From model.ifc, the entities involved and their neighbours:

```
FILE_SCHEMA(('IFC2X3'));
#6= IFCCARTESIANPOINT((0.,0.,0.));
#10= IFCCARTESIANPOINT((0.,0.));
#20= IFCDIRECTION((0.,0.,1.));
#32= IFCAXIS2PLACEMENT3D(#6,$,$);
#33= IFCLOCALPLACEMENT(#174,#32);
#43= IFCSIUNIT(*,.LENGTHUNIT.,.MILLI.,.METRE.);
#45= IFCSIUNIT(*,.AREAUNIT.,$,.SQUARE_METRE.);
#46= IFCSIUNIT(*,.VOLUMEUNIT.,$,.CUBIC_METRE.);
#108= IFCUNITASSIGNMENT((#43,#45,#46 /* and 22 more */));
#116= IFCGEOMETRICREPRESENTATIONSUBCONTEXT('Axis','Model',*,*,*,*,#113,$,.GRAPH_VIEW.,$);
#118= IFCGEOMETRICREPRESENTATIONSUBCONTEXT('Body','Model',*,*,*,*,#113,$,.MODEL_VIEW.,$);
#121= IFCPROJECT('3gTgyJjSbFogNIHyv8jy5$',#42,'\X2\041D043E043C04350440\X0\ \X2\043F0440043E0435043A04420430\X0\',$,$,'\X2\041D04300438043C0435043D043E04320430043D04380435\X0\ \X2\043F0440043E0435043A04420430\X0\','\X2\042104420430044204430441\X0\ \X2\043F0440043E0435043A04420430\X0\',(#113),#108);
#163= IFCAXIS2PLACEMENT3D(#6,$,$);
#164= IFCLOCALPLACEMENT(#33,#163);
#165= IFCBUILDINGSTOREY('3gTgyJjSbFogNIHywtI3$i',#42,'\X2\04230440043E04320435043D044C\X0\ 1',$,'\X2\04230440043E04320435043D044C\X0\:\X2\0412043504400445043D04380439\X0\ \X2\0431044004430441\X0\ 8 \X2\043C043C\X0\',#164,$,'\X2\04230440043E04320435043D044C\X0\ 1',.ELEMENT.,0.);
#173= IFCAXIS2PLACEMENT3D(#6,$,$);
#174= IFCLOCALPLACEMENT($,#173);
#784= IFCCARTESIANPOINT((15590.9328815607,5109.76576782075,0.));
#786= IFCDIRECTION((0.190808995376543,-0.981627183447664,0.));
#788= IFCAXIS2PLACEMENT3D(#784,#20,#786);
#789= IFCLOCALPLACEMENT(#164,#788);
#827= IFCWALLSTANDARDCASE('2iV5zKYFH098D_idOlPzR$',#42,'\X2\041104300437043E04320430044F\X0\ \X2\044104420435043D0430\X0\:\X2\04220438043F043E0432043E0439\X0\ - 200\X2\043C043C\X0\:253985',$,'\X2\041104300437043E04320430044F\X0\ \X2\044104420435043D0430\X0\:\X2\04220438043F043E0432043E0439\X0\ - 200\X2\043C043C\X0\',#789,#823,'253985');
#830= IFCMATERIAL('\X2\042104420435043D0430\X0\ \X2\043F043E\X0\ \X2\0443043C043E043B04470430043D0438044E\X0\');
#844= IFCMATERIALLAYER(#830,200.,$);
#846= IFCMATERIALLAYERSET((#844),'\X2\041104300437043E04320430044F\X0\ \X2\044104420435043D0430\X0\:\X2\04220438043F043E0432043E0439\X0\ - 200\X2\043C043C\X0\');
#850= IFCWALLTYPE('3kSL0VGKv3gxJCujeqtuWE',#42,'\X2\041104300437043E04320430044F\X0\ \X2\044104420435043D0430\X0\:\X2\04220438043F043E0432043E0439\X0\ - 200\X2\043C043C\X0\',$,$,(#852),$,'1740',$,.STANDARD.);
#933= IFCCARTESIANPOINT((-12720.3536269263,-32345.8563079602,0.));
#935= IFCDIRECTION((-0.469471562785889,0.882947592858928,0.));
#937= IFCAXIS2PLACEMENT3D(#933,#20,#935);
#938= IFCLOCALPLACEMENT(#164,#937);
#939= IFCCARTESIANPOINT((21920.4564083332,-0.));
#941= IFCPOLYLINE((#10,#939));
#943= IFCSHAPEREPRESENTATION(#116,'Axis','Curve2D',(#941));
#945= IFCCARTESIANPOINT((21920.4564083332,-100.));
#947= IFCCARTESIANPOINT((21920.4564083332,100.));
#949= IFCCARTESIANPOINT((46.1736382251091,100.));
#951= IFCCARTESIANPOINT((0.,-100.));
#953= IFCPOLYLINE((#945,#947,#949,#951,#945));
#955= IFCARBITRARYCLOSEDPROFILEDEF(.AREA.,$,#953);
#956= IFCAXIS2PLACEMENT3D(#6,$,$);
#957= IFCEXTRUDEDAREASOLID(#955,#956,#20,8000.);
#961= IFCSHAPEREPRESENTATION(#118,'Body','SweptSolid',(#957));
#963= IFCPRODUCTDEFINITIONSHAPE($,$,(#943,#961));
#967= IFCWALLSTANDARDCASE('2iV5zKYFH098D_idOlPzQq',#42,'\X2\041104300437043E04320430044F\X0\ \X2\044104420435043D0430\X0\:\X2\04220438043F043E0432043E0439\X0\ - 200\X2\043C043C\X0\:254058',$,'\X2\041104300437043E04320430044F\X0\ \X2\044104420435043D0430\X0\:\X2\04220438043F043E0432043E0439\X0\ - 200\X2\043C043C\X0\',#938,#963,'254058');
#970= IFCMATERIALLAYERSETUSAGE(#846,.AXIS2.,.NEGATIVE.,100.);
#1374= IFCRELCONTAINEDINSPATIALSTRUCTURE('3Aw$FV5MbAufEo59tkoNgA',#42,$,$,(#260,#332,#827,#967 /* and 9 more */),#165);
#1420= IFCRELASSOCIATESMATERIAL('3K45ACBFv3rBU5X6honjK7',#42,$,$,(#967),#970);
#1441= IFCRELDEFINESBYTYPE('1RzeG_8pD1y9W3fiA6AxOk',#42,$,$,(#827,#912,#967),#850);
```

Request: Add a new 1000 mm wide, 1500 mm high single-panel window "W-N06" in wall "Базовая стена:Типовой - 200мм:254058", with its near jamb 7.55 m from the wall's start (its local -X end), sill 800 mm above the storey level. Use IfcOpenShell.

```python
import numpy as np
import ifcopenshell
import ifcopenshell.api.feature
import ifcopenshell.api.geometry
import ifcopenshell.api.root
import ifcopenshell.api.spatial
import ifcopenshell.api.type
import ifcopenshell.geom
import ifcopenshell.util.element
import ifcopenshell.util.placement
import ifcopenshell.util.representation
import ifcopenshell.util.shape
import ifcopenshell.util.unit

model = ifcopenshell.open("model.ifc")
unit_scale = ifcopenshell.util.unit.calculate_unit_scale(model)
settings = ifcopenshell.geom.settings()


def volume(element):
    """Net volume in cubic metres, openings subtracted."""
    shape = ifcopenshell.geom.create_shape(settings, element)
    return ifcopenshell.util.shape.get_volume(shape.geometry)


wall = model.by_guid("2iV5zKYFH098D_idOlPzQq")
storey = ifcopenshell.util.element.get_container(wall, ifc_class="IfcBuildingStorey")
context = ifcopenshell.util.representation.get_context(model, "Model", "Body", "MODEL_VIEW")
before = volume(wall)

width, height, from_end, sill = 1, 1.5, 7.55, 0.8  # metres

# The wall runs along its own X axis, and the end named is its -X end.
wall_shape = ifcopenshell.geom.create_shape(settings, wall)
x, y, z = ifcopenshell.util.shape.get_vertices(wall_shape.geometry).T
start = x.min() + from_end
face, thickness = float(y.min()), float(y.max() - y.min())
wall_matrix = ifcopenshell.util.placement.get_local_placement(wall.ObjectPlacement)
level = ifcopenshell.util.placement.get_local_placement(storey.ObjectPlacement)[2, 3]


def in_wall(x, y):
    """Placement at x, y metres in the wall's axes, at sill height."""
    matrix = wall_matrix.copy()
    matrix[:, 3] = wall_matrix @ np.array([x / unit_scale, y / unit_scale, 0.0, 1.0])
    matrix[2, 3] = level + sill / unit_scale
    return matrix


# Opening: a box that overshoots both wall faces by 50 mm.
opening = ifcopenshell.api.root.create_entity(model, ifc_class="IfcOpeningElement")
box = ifcopenshell.api.geometry.add_wall_representation(
    model, context=context, length=width, height=height, thickness=thickness + 0.1
)
ifcopenshell.api.geometry.assign_representation(model, product=opening, representation=box)
ifcopenshell.api.geometry.edit_object_placement(model, product=opening, matrix=in_wall(start, face - 0.05), is_si=False)
ifcopenshell.api.feature.add_feature(model, feature=opening, element=wall)

window = ifcopenshell.api.root.create_entity(model, ifc_class="IfcWindow", name="W-N06")
window.OverallWidth, window.OverallHeight = width / unit_scale, height / unit_scale
body = ifcopenshell.api.geometry.add_window_representation(
    model,
    context=context,
    overall_width=window.OverallWidth,
    overall_height=window.OverallHeight,
    partition_type="SINGLE_PANEL",
)
ifcopenshell.api.geometry.assign_representation(model, product=window, representation=body)
ifcopenshell.api.spatial.assign_container(model, products=[window], relating_structure=storey)
fills = ifcopenshell.api.feature.add_filling(model, opening=opening, element=window)
fills.OwnerHistory = window.OwnerHistory  # required in IFC2X3

# IFC2X3 keeps the operation on the window style.
style = ifcopenshell.api.root.create_entity(model, ifc_class="IfcWindowStyle", name="W-N06")
style.OperationType, style.ConstructionType = "SINGLE_PANEL", "NOTDEFINED"
style.ParameterTakesPrecedence = style.Sizeable = False
ifcopenshell.api.type.assign_type(model, related_objects=[window], relating_type=style)

# Centre the window in the wall's thickness.
ifcopenshell.api.geometry.edit_object_placement(model, product=window, matrix=in_wall(start, face), is_si=False)
window_shape = ifcopenshell.geom.create_shape(settings, window)
depth = ifcopenshell.util.shape.get_vertices(window_shape.geometry)[:, 1]
offset = face + thickness / 2 - (depth.min() + depth.max()) / 2
ifcopenshell.api.geometry.edit_object_placement(model, product=window, matrix=in_wall(start, offset), is_si=False)

after = volume(wall)

print(f"wall volume {before:.3f} -> {after:.3f} m3")

model.write("model_edited.ifc")
```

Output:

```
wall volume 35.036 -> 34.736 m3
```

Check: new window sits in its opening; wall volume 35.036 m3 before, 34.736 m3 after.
